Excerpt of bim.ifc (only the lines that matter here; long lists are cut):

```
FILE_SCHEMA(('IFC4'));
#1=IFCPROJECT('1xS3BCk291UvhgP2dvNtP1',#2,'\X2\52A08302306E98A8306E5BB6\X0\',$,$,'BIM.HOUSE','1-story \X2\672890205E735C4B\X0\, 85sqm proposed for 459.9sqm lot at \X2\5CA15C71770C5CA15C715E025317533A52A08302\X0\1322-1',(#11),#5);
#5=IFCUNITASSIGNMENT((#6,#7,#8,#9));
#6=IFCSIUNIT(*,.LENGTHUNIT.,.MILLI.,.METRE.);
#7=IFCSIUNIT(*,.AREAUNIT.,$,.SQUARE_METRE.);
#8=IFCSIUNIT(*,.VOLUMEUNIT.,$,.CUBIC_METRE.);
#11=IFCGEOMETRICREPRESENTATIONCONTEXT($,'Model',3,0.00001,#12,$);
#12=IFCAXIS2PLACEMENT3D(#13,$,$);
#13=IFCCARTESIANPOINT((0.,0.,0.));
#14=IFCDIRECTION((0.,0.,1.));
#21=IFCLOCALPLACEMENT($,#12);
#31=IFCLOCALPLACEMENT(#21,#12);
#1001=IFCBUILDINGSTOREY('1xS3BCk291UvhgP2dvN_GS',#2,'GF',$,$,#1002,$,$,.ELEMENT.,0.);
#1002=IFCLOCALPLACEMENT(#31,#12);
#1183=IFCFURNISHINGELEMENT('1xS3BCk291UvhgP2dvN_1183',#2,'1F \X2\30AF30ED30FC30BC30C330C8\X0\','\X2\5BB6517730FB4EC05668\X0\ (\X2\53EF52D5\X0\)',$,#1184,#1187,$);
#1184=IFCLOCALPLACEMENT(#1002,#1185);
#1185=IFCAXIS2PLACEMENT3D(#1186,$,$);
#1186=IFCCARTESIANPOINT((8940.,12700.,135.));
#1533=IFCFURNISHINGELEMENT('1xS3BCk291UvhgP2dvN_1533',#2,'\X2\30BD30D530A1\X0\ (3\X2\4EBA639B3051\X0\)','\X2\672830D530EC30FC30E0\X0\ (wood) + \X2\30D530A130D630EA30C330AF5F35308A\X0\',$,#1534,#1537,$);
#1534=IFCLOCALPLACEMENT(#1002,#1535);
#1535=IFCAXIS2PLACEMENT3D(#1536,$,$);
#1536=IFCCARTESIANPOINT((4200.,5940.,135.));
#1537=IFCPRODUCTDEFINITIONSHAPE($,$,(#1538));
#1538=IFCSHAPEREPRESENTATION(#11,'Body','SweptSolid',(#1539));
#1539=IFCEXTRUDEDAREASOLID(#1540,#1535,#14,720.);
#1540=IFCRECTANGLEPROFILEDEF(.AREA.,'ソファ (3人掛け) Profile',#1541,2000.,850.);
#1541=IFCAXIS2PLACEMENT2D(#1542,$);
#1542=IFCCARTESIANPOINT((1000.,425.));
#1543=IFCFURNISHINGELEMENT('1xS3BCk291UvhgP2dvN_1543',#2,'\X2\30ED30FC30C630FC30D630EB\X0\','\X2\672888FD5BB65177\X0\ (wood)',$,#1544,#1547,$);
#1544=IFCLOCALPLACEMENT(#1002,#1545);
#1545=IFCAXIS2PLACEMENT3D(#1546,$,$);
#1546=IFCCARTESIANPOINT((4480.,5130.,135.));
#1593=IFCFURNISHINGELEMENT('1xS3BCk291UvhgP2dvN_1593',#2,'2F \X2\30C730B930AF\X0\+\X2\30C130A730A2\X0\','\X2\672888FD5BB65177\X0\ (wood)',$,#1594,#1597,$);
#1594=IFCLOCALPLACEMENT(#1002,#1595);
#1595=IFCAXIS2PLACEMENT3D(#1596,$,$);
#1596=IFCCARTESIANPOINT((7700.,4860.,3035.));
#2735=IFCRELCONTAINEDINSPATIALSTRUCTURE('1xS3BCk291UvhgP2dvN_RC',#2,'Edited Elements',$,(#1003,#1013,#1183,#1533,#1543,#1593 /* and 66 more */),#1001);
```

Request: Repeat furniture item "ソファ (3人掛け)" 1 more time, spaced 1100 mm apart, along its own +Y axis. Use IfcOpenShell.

```python
import ifcopenshell
import ifcopenshell.api.geometry
import ifcopenshell.api.root
import ifcopenshell.util.element
import ifcopenshell.util.placement
import ifcopenshell.util.unit

model = ifcopenshell.open("bim.ifc")
unit_scale = ifcopenshell.util.unit.calculate_unit_scale(model)


def reuse_history(source, copy):
    """copy_class also copies each property set's owner history, people and application; keep the originals."""
    for rel in copy.IsDefinedBy:
        if rel.is_a("IfcRelDefinesByProperties") and (history := rel.RelatingPropertyDefinition.OwnerHistory):
            rel.RelatingPropertyDefinition.OwnerHistory = source.OwnerHistory
            ifcopenshell.util.element.remove_deep2(model, history)


source = model.by_guid("1xS3BCk291UvhgP2dvN_1533")
base = ifcopenshell.util.placement.get_local_placement(source.ObjectPlacement)
step = base[:3, 1] * 1.1 / unit_scale

for i in range(1, 2):
    copy = ifcopenshell.api.root.copy_class(model, product=source)
    copy.Representation = ifcopenshell.util.element.copy_deep(
        model, source.Representation, exclude=["IfcGeometricRepresentationContext", "IfcRepresentationMap"]
    )
    reuse_history(source, copy)
    matrix = base.copy()
    matrix[:3, 3] += i * step
    print("added at", matrix[:3, 3].round(3) + 0.0)
    ifcopenshell.api.geometry.edit_object_placement(model, product=copy, matrix=matrix, is_si=False)

model.write("bim_v2.ifc")
```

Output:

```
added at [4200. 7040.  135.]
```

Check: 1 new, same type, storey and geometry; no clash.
